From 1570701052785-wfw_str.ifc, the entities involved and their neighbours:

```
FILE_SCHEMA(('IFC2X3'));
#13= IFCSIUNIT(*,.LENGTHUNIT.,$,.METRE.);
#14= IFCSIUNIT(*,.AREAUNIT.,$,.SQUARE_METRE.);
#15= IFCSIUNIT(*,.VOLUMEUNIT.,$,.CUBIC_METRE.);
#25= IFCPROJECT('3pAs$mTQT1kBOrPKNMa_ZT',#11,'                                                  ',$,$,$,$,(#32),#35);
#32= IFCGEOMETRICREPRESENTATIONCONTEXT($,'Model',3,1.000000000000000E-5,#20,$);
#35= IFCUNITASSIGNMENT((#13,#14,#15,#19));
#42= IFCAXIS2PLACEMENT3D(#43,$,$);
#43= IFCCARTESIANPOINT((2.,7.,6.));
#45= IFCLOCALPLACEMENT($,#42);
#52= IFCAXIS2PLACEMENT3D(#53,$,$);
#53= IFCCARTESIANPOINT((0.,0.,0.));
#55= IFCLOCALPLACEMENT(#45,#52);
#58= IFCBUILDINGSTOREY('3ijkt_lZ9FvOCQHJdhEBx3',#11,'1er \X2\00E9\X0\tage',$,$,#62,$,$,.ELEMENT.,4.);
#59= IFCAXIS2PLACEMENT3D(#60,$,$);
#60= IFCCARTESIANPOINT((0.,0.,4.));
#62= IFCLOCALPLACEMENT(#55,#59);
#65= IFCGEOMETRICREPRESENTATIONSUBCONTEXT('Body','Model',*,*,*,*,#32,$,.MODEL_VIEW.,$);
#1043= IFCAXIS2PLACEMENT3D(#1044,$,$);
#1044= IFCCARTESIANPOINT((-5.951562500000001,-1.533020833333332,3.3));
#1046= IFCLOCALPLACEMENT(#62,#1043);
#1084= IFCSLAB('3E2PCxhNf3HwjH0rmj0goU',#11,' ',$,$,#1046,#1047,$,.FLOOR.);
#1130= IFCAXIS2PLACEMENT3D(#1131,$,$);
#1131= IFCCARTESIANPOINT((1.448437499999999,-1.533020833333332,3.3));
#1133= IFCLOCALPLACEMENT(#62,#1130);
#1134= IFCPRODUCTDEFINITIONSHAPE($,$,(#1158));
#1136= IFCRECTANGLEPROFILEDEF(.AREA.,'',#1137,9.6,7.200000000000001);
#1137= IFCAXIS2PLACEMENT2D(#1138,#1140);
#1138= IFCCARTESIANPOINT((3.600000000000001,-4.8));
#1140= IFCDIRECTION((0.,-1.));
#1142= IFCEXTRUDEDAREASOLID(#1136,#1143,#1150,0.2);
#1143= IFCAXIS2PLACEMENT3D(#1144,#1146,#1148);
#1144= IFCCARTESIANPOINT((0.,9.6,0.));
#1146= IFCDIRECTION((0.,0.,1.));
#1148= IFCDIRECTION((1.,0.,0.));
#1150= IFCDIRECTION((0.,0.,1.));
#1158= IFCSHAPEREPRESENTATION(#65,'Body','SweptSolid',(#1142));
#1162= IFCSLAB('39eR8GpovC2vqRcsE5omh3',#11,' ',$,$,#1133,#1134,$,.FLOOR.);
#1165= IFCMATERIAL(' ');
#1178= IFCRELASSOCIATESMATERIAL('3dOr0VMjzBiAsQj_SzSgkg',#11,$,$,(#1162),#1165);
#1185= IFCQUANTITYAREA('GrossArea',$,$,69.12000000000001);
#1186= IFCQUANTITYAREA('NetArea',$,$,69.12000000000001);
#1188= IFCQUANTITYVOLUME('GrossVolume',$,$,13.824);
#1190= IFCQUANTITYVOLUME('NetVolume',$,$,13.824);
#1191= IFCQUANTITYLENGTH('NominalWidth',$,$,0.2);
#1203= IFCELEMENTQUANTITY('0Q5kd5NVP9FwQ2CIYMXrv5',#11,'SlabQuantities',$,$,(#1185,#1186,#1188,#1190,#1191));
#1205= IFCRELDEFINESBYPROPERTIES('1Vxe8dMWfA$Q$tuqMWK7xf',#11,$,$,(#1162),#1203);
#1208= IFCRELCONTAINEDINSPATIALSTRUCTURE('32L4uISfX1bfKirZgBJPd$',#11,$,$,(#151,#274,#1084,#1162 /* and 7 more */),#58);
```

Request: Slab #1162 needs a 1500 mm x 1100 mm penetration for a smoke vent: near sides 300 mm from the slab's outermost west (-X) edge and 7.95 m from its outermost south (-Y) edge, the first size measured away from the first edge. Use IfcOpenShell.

```python
import numpy as np
import ifcopenshell
import ifcopenshell.api.feature
import ifcopenshell.api.geometry
import ifcopenshell.api.pset
import ifcopenshell.api.root
import ifcopenshell.geom
import ifcopenshell.util.element
import ifcopenshell.util.placement
import ifcopenshell.util.representation
import ifcopenshell.util.shape
import ifcopenshell.util.unit

model = ifcopenshell.open("1570701052785-wfw_str.ifc")
unit_scale = ifcopenshell.util.unit.calculate_unit_scale(model)
area_scale = ifcopenshell.util.unit.calculate_unit_scale(model, "AREAUNIT")
volume_scale = ifcopenshell.util.unit.calculate_unit_scale(model, "VOLUMEUNIT")
settings = ifcopenshell.geom.settings()


def volume(element):
    """Net volume in cubic metres, openings subtracted."""
    shape = ifcopenshell.geom.create_shape(settings, element)
    return ifcopenshell.util.shape.get_volume(shape.geometry)


slab = model.by_guid("39eR8GpovC2vqRcsE5omh3")
before = volume(slab)

# Extent in the slab's own axes, in metres. The edges named are its -X and -Y sides.
slab_shape = ifcopenshell.geom.create_shape(settings, slab)
vertices = ifcopenshell.util.shape.get_vertices(slab_shape.geometry)
x_min, y_min, bottom = vertices.min(axis=0)
top = vertices[:, 2].max()

opening = ifcopenshell.api.root.create_entity(model, ifc_class="IfcOpeningElement", name="Smoke vent opening")
context = ifcopenshell.util.representation.get_context(model, "Model", "Body", "MODEL_VIEW")
width, depth = 1.5, 1.1
outline = [(0.0, 0.0), (width, 0.0), (width, depth), (0.0, depth), (0.0, 0.0)]
# Overshoot both faces by 50 mm so the cut is clean.
shape = ifcopenshell.api.geometry.add_slab_representation(
    model, context=context, depth=top - bottom + 0.1, polyline=outline
)
ifcopenshell.api.geometry.assign_representation(model, product=opening, representation=shape)

matrix = ifcopenshell.util.placement.get_local_placement(slab.ObjectPlacement)
matrix[:, 3] = matrix @ np.append(np.array([x_min + 0.3, y_min + 7.95, bottom - 0.05]) / unit_scale, 1.0)
ifcopenshell.api.geometry.edit_object_placement(model, product=opening, matrix=matrix, is_si=False)
ifcopenshell.api.feature.add_feature(model, feature=opening, element=slab)

after = volume(slab)

# Update the slab's stored quantities.
qto = model.by_id(ifcopenshell.util.element.get_pset(slab, "SlabQuantities", should_inherit=False)["id"])
ifcopenshell.api.pset.edit_qto(model, qto=qto, properties={
    "NetArea": after / (top - bottom) / area_scale,
    "NetVolume": after / volume_scale,
})

print(f"slab volume {before:.3f} -> {after:.3f} m3")

model.write("1570701052785-wfw_str_v2.ifc")
```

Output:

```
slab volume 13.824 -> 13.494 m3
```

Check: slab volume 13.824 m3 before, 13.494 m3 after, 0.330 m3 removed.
